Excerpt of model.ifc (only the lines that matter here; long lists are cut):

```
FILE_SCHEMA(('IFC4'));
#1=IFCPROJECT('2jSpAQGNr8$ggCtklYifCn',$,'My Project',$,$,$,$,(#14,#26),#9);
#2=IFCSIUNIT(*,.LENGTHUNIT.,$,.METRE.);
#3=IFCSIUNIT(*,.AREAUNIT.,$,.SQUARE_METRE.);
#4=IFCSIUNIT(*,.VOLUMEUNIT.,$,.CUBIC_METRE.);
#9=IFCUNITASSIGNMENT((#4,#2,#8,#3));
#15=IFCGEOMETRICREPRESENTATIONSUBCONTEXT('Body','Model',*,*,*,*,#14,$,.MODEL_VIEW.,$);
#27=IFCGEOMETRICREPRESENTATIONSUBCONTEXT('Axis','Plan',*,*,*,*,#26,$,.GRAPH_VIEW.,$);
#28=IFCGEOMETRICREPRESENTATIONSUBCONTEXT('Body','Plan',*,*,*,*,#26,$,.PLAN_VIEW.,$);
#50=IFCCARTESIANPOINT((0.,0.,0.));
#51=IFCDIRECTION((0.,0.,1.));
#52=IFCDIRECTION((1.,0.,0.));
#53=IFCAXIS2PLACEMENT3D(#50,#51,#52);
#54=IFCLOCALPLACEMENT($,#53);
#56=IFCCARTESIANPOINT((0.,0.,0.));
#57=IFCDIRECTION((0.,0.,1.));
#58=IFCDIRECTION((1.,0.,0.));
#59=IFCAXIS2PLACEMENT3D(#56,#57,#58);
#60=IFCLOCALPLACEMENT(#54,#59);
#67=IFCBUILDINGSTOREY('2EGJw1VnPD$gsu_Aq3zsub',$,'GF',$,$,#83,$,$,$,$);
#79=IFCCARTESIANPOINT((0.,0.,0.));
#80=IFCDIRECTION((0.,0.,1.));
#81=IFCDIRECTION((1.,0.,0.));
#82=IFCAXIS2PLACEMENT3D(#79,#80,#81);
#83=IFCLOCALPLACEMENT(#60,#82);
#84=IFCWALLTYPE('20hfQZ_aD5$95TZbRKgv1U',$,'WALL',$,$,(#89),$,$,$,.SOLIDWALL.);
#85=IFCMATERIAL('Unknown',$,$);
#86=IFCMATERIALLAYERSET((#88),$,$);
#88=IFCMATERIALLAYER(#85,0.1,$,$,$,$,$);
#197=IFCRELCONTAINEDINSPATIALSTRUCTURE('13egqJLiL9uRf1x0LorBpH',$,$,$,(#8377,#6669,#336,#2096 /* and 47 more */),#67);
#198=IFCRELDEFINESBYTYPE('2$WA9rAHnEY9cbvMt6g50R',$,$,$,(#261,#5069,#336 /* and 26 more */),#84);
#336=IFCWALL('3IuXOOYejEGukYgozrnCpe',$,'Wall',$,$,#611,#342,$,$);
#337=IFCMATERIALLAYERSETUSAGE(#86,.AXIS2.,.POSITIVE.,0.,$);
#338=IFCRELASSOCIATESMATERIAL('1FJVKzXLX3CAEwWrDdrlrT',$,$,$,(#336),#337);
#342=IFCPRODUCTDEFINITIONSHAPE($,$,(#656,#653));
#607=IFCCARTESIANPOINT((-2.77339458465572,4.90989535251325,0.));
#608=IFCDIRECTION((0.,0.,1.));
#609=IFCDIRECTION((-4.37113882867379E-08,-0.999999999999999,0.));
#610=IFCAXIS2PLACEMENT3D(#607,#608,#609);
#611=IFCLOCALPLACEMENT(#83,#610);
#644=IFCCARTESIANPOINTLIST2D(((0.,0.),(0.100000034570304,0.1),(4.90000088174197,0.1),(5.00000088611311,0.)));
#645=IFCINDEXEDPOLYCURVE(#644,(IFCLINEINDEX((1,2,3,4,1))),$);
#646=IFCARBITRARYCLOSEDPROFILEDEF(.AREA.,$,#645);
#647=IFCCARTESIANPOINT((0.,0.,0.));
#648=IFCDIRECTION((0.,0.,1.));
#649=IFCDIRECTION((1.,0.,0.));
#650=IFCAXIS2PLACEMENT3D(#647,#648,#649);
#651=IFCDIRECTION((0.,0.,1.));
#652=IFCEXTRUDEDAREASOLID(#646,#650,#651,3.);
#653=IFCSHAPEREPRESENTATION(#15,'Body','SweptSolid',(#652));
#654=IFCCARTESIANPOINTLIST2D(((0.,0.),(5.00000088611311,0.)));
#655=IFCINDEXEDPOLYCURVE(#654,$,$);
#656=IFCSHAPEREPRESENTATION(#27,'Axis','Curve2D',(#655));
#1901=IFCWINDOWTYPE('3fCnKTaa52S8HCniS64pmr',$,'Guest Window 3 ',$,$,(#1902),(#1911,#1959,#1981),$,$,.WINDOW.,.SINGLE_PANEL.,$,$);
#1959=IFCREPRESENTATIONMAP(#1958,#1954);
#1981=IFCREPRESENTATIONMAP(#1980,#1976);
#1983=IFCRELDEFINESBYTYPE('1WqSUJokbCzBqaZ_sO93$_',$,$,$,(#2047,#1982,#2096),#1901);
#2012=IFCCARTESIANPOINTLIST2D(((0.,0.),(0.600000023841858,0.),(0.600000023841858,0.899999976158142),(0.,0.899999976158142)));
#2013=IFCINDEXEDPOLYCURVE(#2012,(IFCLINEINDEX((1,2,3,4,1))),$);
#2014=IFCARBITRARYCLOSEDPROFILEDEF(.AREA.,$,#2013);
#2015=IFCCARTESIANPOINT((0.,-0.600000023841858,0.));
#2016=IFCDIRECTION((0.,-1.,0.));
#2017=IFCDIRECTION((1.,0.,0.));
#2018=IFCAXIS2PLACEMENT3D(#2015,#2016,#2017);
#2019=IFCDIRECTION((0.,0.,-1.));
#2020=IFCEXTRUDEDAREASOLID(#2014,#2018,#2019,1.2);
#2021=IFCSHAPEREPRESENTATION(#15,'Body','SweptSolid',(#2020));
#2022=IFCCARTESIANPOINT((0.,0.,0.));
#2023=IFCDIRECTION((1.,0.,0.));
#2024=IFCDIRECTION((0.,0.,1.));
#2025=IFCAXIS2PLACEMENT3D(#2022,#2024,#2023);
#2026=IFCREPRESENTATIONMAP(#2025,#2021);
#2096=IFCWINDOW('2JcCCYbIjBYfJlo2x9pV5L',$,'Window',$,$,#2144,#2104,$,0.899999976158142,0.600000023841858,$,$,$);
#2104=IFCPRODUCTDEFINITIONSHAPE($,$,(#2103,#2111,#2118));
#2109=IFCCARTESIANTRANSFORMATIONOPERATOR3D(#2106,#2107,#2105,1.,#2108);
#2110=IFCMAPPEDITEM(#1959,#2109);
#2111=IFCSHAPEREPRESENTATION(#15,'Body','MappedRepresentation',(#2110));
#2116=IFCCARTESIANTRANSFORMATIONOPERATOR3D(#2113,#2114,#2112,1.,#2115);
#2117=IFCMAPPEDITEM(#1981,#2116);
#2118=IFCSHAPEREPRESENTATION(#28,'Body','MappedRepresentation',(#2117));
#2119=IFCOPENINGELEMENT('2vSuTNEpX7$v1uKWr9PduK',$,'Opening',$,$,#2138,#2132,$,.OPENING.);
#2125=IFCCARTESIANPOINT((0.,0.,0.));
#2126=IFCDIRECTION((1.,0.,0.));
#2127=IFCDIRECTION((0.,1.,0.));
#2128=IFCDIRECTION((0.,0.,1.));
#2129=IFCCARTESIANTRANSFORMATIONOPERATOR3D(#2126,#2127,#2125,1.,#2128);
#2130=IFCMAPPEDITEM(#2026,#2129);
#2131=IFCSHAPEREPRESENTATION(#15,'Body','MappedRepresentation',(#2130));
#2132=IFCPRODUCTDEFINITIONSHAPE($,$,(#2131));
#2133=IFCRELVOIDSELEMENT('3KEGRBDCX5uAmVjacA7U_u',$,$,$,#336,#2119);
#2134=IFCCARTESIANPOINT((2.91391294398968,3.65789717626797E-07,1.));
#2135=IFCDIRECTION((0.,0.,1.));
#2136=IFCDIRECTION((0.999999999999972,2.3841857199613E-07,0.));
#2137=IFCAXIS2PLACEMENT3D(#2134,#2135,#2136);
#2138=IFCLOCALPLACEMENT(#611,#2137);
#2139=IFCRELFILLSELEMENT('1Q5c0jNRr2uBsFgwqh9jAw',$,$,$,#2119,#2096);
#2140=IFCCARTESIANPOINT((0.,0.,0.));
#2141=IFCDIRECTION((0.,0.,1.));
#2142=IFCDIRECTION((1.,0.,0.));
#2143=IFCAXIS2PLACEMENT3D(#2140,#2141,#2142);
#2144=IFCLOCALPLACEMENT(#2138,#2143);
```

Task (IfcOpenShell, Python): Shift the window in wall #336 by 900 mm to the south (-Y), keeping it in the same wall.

```python
import ifcopenshell
import ifcopenshell.api.geometry
import ifcopenshell.util.placement
import ifcopenshell.util.unit

model = ifcopenshell.open("model.ifc")
unit_scale = ifcopenshell.util.unit.calculate_unit_scale(model)

window = model.by_guid("2JcCCYbIjBYfJlo2x9pV5L")
opening = window.FillsVoids[0].RelatingOpeningElement
wall = opening.VoidsElements[0].RelatingBuildingElement

wall_matrix = ifcopenshell.util.placement.get_local_placement(wall.ObjectPlacement)
shift = wall_matrix[:3, 0] * 0.9 / unit_scale
before = ifcopenshell.util.placement.get_local_placement(window.ObjectPlacement)[:3, 3].copy()

# The window is placed relative to its opening, so it follows when the opening moves.
matrix = ifcopenshell.util.placement.get_local_placement(opening.ObjectPlacement)
matrix[:3, 3] += shift
ifcopenshell.api.geometry.edit_object_placement(
    model, product=opening, matrix=matrix, is_si=False, should_transform_children=True
)

after = ifcopenshell.util.placement.get_local_placement(window.ObjectPlacement)[:3, 3]
print("window moved by", (after - before).round(3) + 0.0)

model.write("model-out.ifc")
```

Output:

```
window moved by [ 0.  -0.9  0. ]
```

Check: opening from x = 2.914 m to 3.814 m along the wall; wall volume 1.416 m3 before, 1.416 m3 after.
